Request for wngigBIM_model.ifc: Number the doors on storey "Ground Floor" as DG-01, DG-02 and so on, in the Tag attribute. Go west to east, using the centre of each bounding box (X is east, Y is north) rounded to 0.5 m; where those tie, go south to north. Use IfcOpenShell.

First a look at what the model holds.

```python
import ifcopenshell
import ifcopenshell.util.element
import ifcopenshell.util.placement

model = ifcopenshell.open("wngigBIM_model.ifc")
print(model.schema)
storey = next(s for s in model.by_type("IfcBuildingStorey") if s.Name == "Ground Floor")
doors = [e for e in ifcopenshell.util.element.get_decomposition(storey) if e.is_a("IfcDoor")]
for e in sorted(doors, key=lambda e: e.id()):
    origin = ifcopenshell.util.placement.get_local_placement(e.ObjectPlacement)[:3, 3]
    print(e.id(), e.Tag, e.Name, origin.round(2) + 0.0, sep=" | ")
```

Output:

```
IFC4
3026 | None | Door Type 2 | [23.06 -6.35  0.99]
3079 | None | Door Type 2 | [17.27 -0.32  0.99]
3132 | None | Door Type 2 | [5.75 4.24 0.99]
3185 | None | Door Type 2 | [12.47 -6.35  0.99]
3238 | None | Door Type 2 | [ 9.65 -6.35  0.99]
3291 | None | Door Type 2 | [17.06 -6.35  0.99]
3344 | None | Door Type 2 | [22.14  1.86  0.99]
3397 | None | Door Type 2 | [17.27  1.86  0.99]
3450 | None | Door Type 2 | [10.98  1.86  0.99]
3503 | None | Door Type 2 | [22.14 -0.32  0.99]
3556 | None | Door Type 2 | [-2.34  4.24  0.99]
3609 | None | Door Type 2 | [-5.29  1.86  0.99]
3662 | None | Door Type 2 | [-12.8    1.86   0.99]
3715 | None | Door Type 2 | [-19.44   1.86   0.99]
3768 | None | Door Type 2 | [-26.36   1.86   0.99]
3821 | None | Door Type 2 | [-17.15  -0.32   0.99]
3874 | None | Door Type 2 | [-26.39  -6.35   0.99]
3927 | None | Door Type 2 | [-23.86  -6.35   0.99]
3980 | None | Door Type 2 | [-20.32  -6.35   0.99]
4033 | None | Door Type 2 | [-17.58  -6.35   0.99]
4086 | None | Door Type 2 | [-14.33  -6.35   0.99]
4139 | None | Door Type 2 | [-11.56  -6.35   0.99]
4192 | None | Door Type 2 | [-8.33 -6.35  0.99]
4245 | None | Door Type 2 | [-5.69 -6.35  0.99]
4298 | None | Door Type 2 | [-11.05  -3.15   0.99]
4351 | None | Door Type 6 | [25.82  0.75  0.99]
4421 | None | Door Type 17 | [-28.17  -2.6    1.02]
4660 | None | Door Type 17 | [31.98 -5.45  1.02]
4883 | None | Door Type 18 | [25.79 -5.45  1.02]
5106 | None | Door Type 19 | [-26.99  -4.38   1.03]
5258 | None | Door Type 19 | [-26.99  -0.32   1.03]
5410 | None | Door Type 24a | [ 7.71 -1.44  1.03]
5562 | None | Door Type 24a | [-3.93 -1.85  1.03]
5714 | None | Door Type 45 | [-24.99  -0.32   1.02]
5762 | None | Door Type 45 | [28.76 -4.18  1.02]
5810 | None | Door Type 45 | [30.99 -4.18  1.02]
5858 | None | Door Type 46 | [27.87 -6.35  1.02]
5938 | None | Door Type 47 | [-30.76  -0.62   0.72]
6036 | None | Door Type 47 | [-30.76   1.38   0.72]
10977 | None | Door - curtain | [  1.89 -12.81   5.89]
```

```python
import ifcopenshell
import ifcopenshell.geom
import ifcopenshell.util.element
import ifcopenshell.util.shape

model = ifcopenshell.open("wngigBIM_model.ifc")
settings = ifcopenshell.geom.settings()
settings.set("use-world-coords", True)


def centre(element):
    shape = ifcopenshell.geom.create_shape(settings, element)
    return ifcopenshell.util.shape.get_bbox_centroid(shape.geometry)


storey = next(s for s in model.by_type("IfcBuildingStorey") if s.Name == "Ground Floor")
doors = [e for e in ifcopenshell.util.element.get_decomposition(storey) if e.is_a("IfcDoor")]

# Insertion points can sit at a corner or the storey origin, so sort by the geometry (in metres).
centres = {e: centre(e) for e in doors}
doors.sort(key=lambda e: (round(centres[e][0] / 0.5), centres[e][1]))

for i, e in enumerate(doors, start=1):
    number = f"DG-{i:02d}"
    e.Tag = number
    print(e.id(), number)

model.write("wngigBIM_model-out.ifc")
```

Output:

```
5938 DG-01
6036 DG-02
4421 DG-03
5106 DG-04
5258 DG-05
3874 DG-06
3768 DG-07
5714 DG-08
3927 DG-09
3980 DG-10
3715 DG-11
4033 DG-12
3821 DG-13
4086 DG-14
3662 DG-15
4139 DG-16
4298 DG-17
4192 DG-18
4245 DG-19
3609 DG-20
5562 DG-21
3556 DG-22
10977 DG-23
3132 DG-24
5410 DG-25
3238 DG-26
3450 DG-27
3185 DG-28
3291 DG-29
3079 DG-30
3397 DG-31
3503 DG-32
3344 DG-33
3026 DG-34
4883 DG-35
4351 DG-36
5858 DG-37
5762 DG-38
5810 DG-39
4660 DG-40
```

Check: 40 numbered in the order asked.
